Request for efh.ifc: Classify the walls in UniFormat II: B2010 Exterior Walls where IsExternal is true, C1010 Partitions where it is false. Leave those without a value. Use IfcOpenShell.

First a look at what the model holds.

```python
import ifcopenshell
import ifcopenshell.util.element

model = ifcopenshell.open("efh.ifc")
print(model.schema)
print("classifications:", [c.Name for c in model.by_type("IfcClassification")])
values = [ifcopenshell.util.element.get_pset(e, "Pset_WallCommon", "IsExternal") for e in model.by_type("IfcWall")]
for value in (True, False, None):
    print("IsExternal", value, values.count(value))
```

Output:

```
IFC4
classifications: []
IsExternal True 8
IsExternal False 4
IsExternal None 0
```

```python
import ifcopenshell
import ifcopenshell.api.classification
import ifcopenshell.util.element

model = ifcopenshell.open("efh.ifc")

system = ifcopenshell.api.classification.add_classification(model, classification="UniFormat II")

walls = model.by_type("IfcWall")
external = {e: ifcopenshell.util.element.get_pset(e, "Pset_WallCommon", "IsExternal") for e in walls}
for flag, code, name in ((True, "B2010", "Exterior Walls"), (False, "C1010", "Partitions")):
    products = [e for e in walls if external[e] is flag]
    ifcopenshell.api.classification.add_reference(
        model, products=products, classification=system, identification=code, name=name
    )
    print(code, len(products))

model.write("efh_v2.ifc")
```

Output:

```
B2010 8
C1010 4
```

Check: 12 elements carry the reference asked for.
